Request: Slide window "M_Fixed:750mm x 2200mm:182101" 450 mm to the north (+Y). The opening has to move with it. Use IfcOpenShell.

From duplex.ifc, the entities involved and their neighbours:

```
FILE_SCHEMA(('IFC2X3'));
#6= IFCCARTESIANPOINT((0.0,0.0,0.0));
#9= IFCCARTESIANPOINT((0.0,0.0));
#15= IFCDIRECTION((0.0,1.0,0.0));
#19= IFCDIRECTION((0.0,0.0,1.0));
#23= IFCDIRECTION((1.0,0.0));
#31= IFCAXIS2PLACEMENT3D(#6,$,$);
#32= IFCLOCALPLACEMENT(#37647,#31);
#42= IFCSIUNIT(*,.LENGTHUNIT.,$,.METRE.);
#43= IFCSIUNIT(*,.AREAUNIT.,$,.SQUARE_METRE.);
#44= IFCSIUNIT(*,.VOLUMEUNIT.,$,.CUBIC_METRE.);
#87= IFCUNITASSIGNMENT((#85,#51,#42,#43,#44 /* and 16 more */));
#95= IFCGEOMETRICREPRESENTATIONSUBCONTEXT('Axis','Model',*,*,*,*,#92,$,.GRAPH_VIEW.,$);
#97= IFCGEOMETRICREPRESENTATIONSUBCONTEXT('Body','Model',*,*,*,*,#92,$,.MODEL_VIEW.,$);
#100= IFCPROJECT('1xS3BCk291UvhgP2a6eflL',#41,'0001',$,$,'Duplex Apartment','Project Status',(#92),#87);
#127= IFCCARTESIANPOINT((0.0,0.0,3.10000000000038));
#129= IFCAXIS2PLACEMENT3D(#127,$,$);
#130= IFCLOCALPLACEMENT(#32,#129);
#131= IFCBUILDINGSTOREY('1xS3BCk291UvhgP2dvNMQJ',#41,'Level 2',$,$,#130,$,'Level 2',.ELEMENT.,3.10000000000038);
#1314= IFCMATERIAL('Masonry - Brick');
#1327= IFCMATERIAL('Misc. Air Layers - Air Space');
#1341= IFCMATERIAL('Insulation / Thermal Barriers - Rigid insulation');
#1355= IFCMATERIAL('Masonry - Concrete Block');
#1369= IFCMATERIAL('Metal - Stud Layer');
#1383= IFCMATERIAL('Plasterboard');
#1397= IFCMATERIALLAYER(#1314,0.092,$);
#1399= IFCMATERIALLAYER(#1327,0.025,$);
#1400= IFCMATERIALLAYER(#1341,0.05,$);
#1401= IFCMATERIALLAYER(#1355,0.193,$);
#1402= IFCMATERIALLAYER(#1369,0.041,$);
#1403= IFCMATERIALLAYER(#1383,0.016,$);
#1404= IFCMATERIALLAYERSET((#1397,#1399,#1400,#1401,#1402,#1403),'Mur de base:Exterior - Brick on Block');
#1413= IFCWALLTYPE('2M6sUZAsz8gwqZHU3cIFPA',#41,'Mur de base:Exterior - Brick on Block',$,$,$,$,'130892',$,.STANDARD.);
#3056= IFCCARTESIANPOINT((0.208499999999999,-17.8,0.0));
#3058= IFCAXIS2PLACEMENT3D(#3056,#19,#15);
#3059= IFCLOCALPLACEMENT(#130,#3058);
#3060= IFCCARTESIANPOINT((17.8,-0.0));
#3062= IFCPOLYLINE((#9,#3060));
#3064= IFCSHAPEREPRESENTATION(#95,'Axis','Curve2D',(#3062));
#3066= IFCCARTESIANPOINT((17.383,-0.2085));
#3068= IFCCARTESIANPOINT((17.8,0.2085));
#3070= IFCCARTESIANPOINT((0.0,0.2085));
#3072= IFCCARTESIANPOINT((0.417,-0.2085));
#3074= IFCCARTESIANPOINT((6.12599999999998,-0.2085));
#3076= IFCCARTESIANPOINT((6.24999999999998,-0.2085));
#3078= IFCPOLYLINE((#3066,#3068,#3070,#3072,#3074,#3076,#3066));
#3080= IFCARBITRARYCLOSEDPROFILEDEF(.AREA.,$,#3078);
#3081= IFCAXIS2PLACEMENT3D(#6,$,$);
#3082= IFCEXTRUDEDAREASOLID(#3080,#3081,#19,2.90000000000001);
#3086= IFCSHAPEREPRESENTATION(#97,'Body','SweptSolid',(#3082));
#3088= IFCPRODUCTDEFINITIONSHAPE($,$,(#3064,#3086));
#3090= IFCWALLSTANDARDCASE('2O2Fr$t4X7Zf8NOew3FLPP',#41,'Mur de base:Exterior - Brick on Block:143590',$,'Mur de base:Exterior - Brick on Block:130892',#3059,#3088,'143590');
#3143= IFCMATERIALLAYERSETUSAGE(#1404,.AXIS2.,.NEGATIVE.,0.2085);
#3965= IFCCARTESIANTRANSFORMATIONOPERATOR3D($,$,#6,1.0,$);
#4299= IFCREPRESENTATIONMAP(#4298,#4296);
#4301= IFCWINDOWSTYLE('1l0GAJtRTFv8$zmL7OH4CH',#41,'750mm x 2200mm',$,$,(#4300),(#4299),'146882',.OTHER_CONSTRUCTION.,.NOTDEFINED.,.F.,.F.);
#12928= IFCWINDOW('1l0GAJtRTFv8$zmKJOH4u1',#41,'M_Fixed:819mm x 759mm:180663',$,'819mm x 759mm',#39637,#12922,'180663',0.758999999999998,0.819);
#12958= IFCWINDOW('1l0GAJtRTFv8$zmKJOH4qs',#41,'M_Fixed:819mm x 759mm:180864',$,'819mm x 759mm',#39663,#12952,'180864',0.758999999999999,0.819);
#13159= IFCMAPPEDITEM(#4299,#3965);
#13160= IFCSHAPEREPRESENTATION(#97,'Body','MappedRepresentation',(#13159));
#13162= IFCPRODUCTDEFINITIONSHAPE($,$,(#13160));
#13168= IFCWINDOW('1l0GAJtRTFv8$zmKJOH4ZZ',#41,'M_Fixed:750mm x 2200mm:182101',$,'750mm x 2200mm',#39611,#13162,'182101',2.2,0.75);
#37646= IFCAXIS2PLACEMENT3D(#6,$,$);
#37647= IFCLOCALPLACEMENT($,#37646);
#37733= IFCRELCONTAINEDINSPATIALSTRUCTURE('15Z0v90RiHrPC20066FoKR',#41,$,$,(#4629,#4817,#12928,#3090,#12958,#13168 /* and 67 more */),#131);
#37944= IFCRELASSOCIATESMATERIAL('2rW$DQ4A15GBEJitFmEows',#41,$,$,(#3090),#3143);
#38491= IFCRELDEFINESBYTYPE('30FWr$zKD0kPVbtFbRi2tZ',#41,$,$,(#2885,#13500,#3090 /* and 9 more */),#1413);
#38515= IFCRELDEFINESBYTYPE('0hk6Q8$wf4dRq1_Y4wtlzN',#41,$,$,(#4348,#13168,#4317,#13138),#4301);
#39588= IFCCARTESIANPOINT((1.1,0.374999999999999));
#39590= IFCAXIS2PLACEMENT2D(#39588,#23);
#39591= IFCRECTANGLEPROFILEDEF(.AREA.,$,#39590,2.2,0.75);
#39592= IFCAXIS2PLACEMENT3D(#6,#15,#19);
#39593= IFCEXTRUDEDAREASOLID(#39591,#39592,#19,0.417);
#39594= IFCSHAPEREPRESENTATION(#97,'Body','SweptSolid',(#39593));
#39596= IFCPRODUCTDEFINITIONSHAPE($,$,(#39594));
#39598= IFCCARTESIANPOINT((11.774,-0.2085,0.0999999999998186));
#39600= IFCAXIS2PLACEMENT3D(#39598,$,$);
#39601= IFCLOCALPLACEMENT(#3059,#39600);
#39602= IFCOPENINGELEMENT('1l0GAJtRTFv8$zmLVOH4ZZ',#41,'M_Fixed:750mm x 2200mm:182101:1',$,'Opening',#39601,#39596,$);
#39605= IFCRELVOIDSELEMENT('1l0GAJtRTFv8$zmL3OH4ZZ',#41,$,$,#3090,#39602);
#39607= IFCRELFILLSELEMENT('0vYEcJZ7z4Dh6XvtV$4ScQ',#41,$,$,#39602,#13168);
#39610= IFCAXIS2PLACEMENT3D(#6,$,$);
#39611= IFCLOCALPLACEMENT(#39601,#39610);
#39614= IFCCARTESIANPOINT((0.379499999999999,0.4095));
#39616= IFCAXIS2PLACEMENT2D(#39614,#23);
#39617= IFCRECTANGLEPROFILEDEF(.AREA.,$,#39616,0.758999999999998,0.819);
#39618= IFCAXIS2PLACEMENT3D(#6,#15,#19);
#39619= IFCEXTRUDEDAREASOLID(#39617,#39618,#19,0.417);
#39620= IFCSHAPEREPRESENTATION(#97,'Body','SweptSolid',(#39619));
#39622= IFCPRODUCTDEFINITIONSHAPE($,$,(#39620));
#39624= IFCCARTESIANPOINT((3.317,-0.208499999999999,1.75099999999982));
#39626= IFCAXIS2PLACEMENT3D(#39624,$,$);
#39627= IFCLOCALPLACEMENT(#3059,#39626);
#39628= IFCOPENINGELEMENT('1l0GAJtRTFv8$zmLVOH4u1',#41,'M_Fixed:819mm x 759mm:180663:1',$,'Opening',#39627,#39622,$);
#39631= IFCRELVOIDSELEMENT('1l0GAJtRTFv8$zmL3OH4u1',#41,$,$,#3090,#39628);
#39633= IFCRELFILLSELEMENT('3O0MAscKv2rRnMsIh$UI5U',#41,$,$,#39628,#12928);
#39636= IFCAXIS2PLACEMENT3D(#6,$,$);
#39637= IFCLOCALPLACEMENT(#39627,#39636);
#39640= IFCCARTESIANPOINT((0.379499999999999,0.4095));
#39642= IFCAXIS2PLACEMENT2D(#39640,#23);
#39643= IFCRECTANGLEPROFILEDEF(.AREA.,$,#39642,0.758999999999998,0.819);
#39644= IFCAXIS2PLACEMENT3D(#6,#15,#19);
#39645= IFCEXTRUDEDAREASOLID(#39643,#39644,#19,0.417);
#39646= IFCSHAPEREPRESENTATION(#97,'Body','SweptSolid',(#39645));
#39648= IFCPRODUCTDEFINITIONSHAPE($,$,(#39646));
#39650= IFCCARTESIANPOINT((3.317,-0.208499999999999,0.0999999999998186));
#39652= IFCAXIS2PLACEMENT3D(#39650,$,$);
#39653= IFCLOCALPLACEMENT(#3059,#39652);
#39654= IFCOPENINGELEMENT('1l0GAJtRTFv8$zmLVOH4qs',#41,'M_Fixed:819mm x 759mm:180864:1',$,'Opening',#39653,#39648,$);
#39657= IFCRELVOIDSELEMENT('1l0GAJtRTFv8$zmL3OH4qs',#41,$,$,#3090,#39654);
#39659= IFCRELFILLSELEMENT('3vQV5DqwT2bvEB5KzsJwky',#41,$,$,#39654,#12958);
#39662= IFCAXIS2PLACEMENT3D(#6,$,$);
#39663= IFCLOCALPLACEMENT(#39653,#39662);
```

```python
import ifcopenshell
import ifcopenshell.api.geometry
import ifcopenshell.util.placement

model = ifcopenshell.open("duplex.ifc")

window = model.by_guid("1l0GAJtRTFv8$zmKJOH4ZZ")
opening = window.FillsVoids[0].RelatingOpeningElement
wall = opening.VoidsElements[0].RelatingBuildingElement

wall_matrix = ifcopenshell.util.placement.get_local_placement(wall.ObjectPlacement)
shift = wall_matrix[:3, 0] * 0.45
before = ifcopenshell.util.placement.get_local_placement(window.ObjectPlacement)[:3, 3].copy()

# The window is placed relative to its opening, so it follows when the opening moves.
matrix = ifcopenshell.util.placement.get_local_placement(opening.ObjectPlacement)
matrix[:3, 3] += shift
ifcopenshell.api.geometry.edit_object_placement(
    model, product=opening, matrix=matrix, is_si=False, should_transform_children=True
)

after = ifcopenshell.util.placement.get_local_placement(window.ObjectPlacement)[:3, 3]
print("window moved by", (after - before).round(3) + 0.0)

model.write("duplex-out.ifc")
```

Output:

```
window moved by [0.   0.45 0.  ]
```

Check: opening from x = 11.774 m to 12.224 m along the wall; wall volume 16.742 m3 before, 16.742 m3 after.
